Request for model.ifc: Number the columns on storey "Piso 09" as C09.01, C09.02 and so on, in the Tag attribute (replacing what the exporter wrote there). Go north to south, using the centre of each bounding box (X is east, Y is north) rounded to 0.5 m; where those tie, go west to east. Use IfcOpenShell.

First a look at what the model holds.

```python
import ifcopenshell
import ifcopenshell.util.element
import ifcopenshell.util.placement

model = ifcopenshell.open("model.ifc")
print(model.schema)
storey = next(s for s in model.by_type("IfcBuildingStorey") if s.Name == "Piso 09")
columns = [e for e in ifcopenshell.util.element.get_decomposition(storey) if e.is_a("IfcColumn")]
for e in sorted(columns, key=lambda e: e.id()):
    origin = ifcopenshell.util.placement.get_local_placement(e.ObjectPlacement)[:3, 3]
    print(e.id(), e.Tag, e.Name, origin.round(2) + 0.0, sep=" | ")
```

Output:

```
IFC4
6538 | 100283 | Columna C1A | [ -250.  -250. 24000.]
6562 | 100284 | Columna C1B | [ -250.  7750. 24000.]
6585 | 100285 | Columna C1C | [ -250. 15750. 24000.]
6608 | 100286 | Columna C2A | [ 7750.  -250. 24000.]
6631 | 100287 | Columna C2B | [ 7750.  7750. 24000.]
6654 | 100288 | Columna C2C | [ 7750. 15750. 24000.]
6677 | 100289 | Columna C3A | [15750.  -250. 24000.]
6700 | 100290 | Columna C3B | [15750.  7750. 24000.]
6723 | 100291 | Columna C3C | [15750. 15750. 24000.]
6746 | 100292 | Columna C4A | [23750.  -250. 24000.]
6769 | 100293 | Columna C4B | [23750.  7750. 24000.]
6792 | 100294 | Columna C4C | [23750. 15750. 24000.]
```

```python
import ifcopenshell
import ifcopenshell.geom
import ifcopenshell.util.element
import ifcopenshell.util.shape

model = ifcopenshell.open("model.ifc")
settings = ifcopenshell.geom.settings()
settings.set("use-world-coords", True)


def centre(element):
    shape = ifcopenshell.geom.create_shape(settings, element)
    return ifcopenshell.util.shape.get_bbox_centroid(shape.geometry)


storey = next(s for s in model.by_type("IfcBuildingStorey") if s.Name == "Piso 09")
columns = [e for e in ifcopenshell.util.element.get_decomposition(storey) if e.is_a("IfcColumn")]

# Insertion points can sit at a corner or the storey origin, so sort by the geometry (in metres).
centres = {e: centre(e) for e in columns}
columns.sort(key=lambda e: (-round(centres[e][1] / 0.5), centres[e][0]))

for i, e in enumerate(columns, start=1):
    number = f"C09.{i:02d}"
    e.Tag = number
    print(e.id(), number)

model.write("model_edited.ifc")
```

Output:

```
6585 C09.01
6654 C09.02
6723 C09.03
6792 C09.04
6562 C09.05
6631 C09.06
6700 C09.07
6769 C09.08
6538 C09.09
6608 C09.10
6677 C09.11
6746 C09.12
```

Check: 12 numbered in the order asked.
